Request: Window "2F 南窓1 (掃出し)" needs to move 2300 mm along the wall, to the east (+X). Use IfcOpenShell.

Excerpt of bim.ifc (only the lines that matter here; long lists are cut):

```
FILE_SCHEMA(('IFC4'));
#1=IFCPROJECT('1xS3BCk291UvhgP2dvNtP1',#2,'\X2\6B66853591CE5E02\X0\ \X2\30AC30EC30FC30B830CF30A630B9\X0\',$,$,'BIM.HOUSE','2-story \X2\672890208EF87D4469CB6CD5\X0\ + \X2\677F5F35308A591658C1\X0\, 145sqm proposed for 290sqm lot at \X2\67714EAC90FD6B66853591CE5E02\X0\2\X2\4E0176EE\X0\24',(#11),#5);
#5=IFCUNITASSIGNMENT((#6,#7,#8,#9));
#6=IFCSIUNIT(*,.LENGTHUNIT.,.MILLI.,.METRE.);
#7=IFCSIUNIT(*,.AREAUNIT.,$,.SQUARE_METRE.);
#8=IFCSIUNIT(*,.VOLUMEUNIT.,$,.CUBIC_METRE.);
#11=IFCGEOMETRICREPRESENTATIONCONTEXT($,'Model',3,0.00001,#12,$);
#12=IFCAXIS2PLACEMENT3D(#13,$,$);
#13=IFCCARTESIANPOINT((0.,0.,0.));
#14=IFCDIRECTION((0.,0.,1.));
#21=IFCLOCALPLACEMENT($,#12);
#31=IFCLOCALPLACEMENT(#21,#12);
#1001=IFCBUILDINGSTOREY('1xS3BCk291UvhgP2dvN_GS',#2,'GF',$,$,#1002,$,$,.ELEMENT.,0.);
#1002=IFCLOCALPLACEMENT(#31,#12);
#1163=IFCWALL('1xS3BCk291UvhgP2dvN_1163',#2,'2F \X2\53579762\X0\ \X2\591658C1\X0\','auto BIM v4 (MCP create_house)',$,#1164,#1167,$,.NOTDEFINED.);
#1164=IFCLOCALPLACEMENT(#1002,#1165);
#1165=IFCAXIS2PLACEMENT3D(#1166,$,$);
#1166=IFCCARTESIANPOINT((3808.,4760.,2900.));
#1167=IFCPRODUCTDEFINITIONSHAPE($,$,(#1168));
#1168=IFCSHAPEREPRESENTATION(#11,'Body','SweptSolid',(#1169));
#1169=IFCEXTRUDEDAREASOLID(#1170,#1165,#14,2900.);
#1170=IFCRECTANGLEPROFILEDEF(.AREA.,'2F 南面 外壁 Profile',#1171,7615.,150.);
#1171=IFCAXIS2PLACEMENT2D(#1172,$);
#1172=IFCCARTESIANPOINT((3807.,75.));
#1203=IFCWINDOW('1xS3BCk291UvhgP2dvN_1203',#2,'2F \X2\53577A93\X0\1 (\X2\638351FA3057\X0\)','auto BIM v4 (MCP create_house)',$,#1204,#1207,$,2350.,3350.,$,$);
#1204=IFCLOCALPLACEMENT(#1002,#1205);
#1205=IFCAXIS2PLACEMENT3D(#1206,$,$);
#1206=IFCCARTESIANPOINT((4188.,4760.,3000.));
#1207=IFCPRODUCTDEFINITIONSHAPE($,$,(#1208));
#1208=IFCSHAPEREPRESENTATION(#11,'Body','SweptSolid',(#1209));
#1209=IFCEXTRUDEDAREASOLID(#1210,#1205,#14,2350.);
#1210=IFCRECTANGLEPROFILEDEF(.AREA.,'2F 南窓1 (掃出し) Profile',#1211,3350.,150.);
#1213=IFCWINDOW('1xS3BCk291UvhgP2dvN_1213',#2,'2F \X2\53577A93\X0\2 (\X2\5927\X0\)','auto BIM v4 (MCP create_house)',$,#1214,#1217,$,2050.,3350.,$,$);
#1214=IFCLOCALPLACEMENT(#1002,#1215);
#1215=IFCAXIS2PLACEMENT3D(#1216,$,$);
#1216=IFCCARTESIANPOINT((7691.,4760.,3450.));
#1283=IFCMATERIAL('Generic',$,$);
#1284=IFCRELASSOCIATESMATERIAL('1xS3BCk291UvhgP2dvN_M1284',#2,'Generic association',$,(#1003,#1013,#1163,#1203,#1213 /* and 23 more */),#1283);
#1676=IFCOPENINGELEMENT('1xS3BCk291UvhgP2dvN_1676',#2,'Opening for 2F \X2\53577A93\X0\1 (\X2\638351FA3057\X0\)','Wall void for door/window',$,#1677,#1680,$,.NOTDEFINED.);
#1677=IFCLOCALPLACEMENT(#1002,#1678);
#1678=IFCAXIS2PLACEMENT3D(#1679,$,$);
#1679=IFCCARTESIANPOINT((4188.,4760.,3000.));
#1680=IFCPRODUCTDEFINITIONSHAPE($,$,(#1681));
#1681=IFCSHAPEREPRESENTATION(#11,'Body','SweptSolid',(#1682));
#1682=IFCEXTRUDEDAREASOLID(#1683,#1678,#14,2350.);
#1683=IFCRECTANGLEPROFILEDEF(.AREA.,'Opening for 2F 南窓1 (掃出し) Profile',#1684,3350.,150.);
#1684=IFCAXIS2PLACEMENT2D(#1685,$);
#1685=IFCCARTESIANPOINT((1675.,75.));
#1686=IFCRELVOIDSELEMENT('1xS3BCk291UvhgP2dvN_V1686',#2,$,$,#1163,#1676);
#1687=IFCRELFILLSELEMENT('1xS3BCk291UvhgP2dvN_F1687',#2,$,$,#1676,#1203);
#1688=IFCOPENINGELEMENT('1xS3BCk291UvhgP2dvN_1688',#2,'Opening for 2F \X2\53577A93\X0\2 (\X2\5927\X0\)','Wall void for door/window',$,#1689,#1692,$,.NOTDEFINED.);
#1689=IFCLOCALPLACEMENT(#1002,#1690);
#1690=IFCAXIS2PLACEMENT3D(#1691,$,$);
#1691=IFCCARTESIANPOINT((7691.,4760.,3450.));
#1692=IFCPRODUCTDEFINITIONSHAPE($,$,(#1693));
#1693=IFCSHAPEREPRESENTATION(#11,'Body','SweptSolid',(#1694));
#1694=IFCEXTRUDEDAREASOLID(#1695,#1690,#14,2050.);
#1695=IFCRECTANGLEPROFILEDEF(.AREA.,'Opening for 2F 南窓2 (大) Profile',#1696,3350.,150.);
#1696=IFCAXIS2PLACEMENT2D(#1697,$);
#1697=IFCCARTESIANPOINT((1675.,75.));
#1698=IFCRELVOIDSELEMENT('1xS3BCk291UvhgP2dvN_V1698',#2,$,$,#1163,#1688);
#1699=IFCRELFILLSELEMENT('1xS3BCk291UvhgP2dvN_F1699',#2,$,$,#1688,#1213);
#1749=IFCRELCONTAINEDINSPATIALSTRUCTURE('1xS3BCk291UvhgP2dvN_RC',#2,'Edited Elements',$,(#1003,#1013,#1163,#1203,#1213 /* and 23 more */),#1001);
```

```python
import ifcopenshell
import ifcopenshell.api.geometry
import ifcopenshell.util.placement
import ifcopenshell.util.unit

model = ifcopenshell.open("bim.ifc")
unit_scale = ifcopenshell.util.unit.calculate_unit_scale(model)

window = model.by_guid("1xS3BCk291UvhgP2dvN_1203")
opening = window.FillsVoids[0].RelatingOpeningElement
wall = opening.VoidsElements[0].RelatingBuildingElement

wall_matrix = ifcopenshell.util.placement.get_local_placement(wall.ObjectPlacement)
shift = wall_matrix[:3, 0] * 2.3 / unit_scale
before = ifcopenshell.util.placement.get_local_placement(window.ObjectPlacement)[:3, 3].copy()

# The window is not placed relative to its opening, so move both.
for product in (opening, window):
    matrix = ifcopenshell.util.placement.get_local_placement(product.ObjectPlacement)
    matrix[:3, 3] += shift
    ifcopenshell.api.geometry.edit_object_placement(model, product=product, matrix=matrix, is_si=False)

after = ifcopenshell.util.placement.get_local_placement(window.ObjectPlacement)[:3, 3]
print("window moved by", (after - before).round(3) + 0.0)

model.write("bim_updated.ifc")
```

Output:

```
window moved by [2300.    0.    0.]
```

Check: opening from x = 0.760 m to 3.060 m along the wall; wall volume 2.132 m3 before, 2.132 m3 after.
